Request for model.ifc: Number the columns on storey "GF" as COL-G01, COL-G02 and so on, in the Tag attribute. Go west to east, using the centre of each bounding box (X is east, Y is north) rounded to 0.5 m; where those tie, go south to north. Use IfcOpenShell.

First a look at what the model holds.

```python
import ifcopenshell
import ifcopenshell.util.element
import ifcopenshell.util.placement

model = ifcopenshell.open("model.ifc")
print(model.schema)
storey = next(s for s in model.by_type("IfcBuildingStorey") if s.Name == "GF")
columns = [e for e in ifcopenshell.util.element.get_decomposition(storey) if e.is_a("IfcColumn")]
for e in sorted(columns, key=lambda e: e.id()):
    origin = ifcopenshell.util.placement.get_local_placement(e.ObjectPlacement)[:3, 3]
    print(e.id(), e.Tag, e.Name, origin.round(2) + 0.0, sep=" | ")
```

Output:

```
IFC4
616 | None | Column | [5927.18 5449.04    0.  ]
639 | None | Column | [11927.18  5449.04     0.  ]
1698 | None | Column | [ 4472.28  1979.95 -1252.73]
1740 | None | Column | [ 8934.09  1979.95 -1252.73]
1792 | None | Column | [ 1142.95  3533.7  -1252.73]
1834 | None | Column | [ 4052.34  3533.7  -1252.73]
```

```python
import ifcopenshell
import ifcopenshell.geom
import ifcopenshell.util.element
import ifcopenshell.util.shape

model = ifcopenshell.open("model.ifc")
settings = ifcopenshell.geom.settings()
settings.set("use-world-coords", True)


def centre(element):
    shape = ifcopenshell.geom.create_shape(settings, element)
    return ifcopenshell.util.shape.get_bbox_centroid(shape.geometry)


storey = next(s for s in model.by_type("IfcBuildingStorey") if s.Name == "GF")
columns = [e for e in ifcopenshell.util.element.get_decomposition(storey) if e.is_a("IfcColumn")]

# Insertion points can sit at a corner or the storey origin, so sort by the geometry (in metres).
centres = {e: centre(e) for e in columns}
columns.sort(key=lambda e: (round(centres[e][0] / 0.5), centres[e][1]))

for i, e in enumerate(columns, start=1):
    number = f"COL-G{i:02d}"
    e.Tag = number
    print(e.id(), number)

model.write("model_edited.ifc")
```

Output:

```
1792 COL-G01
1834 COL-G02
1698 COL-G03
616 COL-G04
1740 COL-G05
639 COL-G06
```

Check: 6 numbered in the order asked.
